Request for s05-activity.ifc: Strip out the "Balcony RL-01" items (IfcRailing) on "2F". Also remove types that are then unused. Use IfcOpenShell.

First a look at what the model holds.

```python
import ifcopenshell
import ifcopenshell.util.element

model = ifcopenshell.open("s05-activity.ifc")
print(model.schema)
storey = next(s for s in model.by_type("IfcBuildingStorey") if s.Name == "2F")
railings = [e for e in ifcopenshell.util.element.get_decomposition(storey) if e.is_a("IfcRailing")]
seen = {}
for e in railings:
    element_type = ifcopenshell.util.element.get_type(e)
    name = element_type.Name if element_type not in (None, e) else None
    seen[name] = seen.get(name, 0) + 1
for name, count in sorted(seen.items(), key=str):
    print(count, "x", name)
```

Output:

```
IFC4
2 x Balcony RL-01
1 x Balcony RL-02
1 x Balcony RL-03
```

```python
import ifcopenshell
import ifcopenshell.api.root
import ifcopenshell.util.element

model = ifcopenshell.open("s05-activity.ifc")

storey = next(s for s in model.by_type("IfcBuildingStorey") if s.Name == "2F")
railings = [e for e in ifcopenshell.util.element.get_decomposition(storey) if e.is_a("IfcRailing")]
targets = [e for e in railings if (t := ifcopenshell.util.element.get_type(e)) not in (None, e) and t.Name == "Balcony RL-01"]
types = {ifcopenshell.util.element.get_type(e) for e in targets} - {None, *targets}

for e in targets:
    ifcopenshell.api.root.remove_product(model, product=e)
print(len(targets), "removed")

unused = [t for t in types if not ifcopenshell.util.element.get_types(t)]
for t in unused:
    ifcopenshell.api.root.remove_product(model, product=t)
print(len(unused), "unused types removed")

model.write("s05-activity_edited.ifc")
```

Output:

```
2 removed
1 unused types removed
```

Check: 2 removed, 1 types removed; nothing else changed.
